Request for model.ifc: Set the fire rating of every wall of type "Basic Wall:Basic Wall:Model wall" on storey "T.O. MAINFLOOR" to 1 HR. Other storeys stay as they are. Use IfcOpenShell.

First a look at what the model holds.

```python
import ifcopenshell
import ifcopenshell.util.element

model = ifcopenshell.open("model.ifc")
print(model.schema)
storey = next(s for s in model.by_type("IfcBuildingStorey") if s.Name == "T.O. MAINFLOOR")
walls = [e for e in ifcopenshell.util.element.get_decomposition(storey) if e.is_a("IfcWall")]
seen = {}
for e in walls:
    element_type = ifcopenshell.util.element.get_type(e)
    key = (element_type.Name if element_type != e and element_type else None, ifcopenshell.util.element.get_pset(e, "Pset_WallCommon", "FireRating"))
    seen[key] = seen.get(key, 0) + 1
for (name, value), count in sorted(seen.items(), key=str):
    print(count, "x", name, "|", value)
```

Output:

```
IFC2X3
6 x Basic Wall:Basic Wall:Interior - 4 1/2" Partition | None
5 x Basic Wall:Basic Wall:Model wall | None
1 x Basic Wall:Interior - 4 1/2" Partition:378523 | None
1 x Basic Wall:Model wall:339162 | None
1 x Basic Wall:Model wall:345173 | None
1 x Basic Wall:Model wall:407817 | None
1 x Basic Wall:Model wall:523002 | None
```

```python
import ifcopenshell
import ifcopenshell.api.pset
import ifcopenshell.util.element

model = ifcopenshell.open("model.ifc")

storey = next(s for s in model.by_type("IfcBuildingStorey") if s.Name == "T.O. MAINFLOOR")
walls = [e for e in ifcopenshell.util.element.get_decomposition(storey) if e.is_a("IfcWall")]

count = 0
for e in walls:
    element_type = ifcopenshell.util.element.get_type(e)
    if element_type in (None, e) or element_type.Name != "Basic Wall:Basic Wall:Model wall":
        continue
    # add_pset returns the element's existing set when there is one.
    pset = ifcopenshell.api.pset.add_pset(model, product=e, name="Pset_WallCommon")
    ifcopenshell.api.pset.edit_pset(model, pset=pset, properties={"FireRating": "1 HR"})
    count += 1

print(count, "walls updated")

model.write("model_updated.ifc")
```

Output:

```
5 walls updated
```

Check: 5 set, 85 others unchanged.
